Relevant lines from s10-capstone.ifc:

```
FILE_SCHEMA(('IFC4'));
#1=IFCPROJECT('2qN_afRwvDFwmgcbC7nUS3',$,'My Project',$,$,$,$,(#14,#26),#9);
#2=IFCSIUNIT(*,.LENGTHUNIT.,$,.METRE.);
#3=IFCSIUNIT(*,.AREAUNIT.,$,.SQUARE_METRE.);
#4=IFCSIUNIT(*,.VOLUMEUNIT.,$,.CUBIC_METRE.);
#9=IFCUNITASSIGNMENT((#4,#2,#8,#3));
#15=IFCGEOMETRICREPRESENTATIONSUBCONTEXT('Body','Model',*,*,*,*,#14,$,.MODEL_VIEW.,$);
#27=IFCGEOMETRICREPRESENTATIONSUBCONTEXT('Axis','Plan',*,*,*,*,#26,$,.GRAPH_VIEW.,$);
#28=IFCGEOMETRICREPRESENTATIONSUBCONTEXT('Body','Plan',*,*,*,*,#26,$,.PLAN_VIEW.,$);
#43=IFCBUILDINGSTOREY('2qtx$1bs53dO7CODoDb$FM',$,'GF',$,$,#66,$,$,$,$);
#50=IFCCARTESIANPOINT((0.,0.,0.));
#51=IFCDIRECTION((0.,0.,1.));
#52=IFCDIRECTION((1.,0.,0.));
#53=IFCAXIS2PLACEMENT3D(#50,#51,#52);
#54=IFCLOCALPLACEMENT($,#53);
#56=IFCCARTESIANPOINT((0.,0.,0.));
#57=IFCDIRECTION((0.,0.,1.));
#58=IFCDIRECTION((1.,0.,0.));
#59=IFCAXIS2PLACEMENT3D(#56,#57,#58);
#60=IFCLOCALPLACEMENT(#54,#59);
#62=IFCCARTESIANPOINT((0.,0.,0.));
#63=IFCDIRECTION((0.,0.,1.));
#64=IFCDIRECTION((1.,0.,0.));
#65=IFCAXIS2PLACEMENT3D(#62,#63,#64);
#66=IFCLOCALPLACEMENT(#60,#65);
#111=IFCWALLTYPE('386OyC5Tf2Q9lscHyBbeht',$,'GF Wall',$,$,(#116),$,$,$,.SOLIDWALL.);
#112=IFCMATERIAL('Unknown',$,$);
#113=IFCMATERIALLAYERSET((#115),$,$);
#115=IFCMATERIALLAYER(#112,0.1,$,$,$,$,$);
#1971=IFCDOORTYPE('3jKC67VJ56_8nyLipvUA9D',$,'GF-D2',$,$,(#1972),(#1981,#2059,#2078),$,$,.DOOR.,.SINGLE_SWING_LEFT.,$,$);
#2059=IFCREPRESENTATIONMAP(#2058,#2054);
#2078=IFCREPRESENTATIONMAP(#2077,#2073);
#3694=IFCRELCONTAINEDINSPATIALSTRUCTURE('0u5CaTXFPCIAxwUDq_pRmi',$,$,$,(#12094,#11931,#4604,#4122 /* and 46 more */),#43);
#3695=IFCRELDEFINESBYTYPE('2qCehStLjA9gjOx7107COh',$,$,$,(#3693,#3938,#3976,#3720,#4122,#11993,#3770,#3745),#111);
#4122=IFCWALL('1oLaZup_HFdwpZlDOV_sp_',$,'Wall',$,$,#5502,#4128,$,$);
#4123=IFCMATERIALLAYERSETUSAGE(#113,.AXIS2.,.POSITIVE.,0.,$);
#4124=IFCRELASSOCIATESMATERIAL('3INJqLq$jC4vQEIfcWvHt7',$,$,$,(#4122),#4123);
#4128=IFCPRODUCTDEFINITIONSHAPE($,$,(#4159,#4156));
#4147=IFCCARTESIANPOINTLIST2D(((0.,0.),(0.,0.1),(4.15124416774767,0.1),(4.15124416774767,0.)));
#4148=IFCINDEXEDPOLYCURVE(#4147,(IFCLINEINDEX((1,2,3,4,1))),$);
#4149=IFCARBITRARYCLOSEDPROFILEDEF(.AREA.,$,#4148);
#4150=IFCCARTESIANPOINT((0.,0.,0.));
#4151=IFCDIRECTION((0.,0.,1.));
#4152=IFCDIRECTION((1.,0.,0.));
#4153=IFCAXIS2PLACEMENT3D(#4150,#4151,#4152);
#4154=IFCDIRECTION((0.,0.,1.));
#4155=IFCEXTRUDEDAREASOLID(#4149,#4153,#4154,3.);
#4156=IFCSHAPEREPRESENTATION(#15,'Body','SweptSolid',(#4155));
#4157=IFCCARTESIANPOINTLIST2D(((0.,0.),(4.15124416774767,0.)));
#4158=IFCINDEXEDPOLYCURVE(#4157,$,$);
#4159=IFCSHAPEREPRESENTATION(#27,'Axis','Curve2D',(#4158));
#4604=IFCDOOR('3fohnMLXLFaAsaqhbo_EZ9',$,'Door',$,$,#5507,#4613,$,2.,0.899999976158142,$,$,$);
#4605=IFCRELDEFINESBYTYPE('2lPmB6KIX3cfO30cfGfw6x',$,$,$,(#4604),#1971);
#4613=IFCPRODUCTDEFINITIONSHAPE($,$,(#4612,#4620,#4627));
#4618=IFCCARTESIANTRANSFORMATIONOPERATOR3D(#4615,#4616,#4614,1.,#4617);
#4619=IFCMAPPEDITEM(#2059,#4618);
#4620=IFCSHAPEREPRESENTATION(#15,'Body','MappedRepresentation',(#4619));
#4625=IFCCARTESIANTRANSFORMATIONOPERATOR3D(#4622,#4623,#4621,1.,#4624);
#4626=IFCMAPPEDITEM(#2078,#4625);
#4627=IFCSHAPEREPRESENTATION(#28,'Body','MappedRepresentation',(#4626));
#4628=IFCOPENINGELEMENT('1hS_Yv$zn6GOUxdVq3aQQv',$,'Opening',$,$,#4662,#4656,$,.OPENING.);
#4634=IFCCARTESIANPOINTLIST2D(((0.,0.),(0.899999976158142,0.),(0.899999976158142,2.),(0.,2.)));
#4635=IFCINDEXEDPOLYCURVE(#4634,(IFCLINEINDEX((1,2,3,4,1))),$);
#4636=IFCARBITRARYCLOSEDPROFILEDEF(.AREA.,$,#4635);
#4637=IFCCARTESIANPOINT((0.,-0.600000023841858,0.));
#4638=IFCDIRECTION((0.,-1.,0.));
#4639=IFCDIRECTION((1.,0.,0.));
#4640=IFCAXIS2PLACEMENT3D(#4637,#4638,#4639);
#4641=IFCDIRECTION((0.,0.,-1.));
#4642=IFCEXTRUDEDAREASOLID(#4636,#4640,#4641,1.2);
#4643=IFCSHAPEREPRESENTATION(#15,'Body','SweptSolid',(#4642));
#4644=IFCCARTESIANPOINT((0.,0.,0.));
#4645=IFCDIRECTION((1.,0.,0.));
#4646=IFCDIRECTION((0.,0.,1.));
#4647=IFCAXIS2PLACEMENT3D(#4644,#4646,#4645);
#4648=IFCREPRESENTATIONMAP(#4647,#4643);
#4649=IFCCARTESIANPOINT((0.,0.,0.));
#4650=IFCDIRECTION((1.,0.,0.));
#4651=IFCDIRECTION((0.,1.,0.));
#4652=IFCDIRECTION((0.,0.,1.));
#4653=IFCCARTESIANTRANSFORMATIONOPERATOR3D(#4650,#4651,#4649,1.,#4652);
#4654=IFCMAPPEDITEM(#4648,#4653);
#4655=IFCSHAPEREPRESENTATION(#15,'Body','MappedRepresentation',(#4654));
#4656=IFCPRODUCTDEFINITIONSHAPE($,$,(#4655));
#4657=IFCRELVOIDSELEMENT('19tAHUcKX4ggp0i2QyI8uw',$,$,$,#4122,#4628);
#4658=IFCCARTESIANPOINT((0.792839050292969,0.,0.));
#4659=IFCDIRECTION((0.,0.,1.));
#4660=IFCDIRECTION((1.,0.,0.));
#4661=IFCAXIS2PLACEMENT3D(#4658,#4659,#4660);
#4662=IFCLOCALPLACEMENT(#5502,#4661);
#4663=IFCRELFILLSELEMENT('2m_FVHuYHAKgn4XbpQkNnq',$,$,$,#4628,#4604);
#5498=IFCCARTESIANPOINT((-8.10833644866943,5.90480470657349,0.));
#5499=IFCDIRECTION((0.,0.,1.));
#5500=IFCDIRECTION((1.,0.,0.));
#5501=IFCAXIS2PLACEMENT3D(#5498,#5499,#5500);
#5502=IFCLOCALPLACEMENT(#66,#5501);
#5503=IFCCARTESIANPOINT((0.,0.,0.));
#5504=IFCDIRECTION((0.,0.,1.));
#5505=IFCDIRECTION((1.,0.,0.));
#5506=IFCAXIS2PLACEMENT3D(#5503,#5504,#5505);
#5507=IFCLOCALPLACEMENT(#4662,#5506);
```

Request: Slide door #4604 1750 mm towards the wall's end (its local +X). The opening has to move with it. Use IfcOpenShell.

```python
import ifcopenshell
import ifcopenshell.api.geometry
import ifcopenshell.util.placement
import ifcopenshell.util.unit

model = ifcopenshell.open("s10-capstone.ifc")
unit_scale = ifcopenshell.util.unit.calculate_unit_scale(model)

door = model.by_guid("3fohnMLXLFaAsaqhbo_EZ9")
opening = door.FillsVoids[0].RelatingOpeningElement
wall = opening.VoidsElements[0].RelatingBuildingElement

wall_matrix = ifcopenshell.util.placement.get_local_placement(wall.ObjectPlacement)
shift = wall_matrix[:3, 0] * 1.75 / unit_scale
before = ifcopenshell.util.placement.get_local_placement(door.ObjectPlacement)[:3, 3].copy()

# The door is placed relative to its opening, so it follows when the opening moves.
matrix = ifcopenshell.util.placement.get_local_placement(opening.ObjectPlacement)
matrix[:3, 3] += shift
ifcopenshell.api.geometry.edit_object_placement(
    model, product=opening, matrix=matrix, is_si=False, should_transform_children=True
)

after = ifcopenshell.util.placement.get_local_placement(door.ObjectPlacement)[:3, 3]
print("door moved by", (after - before).round(3) + 0.0)

model.write("s10-capstone_edited.ifc")
```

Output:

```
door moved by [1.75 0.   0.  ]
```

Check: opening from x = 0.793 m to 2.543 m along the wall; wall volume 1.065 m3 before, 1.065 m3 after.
